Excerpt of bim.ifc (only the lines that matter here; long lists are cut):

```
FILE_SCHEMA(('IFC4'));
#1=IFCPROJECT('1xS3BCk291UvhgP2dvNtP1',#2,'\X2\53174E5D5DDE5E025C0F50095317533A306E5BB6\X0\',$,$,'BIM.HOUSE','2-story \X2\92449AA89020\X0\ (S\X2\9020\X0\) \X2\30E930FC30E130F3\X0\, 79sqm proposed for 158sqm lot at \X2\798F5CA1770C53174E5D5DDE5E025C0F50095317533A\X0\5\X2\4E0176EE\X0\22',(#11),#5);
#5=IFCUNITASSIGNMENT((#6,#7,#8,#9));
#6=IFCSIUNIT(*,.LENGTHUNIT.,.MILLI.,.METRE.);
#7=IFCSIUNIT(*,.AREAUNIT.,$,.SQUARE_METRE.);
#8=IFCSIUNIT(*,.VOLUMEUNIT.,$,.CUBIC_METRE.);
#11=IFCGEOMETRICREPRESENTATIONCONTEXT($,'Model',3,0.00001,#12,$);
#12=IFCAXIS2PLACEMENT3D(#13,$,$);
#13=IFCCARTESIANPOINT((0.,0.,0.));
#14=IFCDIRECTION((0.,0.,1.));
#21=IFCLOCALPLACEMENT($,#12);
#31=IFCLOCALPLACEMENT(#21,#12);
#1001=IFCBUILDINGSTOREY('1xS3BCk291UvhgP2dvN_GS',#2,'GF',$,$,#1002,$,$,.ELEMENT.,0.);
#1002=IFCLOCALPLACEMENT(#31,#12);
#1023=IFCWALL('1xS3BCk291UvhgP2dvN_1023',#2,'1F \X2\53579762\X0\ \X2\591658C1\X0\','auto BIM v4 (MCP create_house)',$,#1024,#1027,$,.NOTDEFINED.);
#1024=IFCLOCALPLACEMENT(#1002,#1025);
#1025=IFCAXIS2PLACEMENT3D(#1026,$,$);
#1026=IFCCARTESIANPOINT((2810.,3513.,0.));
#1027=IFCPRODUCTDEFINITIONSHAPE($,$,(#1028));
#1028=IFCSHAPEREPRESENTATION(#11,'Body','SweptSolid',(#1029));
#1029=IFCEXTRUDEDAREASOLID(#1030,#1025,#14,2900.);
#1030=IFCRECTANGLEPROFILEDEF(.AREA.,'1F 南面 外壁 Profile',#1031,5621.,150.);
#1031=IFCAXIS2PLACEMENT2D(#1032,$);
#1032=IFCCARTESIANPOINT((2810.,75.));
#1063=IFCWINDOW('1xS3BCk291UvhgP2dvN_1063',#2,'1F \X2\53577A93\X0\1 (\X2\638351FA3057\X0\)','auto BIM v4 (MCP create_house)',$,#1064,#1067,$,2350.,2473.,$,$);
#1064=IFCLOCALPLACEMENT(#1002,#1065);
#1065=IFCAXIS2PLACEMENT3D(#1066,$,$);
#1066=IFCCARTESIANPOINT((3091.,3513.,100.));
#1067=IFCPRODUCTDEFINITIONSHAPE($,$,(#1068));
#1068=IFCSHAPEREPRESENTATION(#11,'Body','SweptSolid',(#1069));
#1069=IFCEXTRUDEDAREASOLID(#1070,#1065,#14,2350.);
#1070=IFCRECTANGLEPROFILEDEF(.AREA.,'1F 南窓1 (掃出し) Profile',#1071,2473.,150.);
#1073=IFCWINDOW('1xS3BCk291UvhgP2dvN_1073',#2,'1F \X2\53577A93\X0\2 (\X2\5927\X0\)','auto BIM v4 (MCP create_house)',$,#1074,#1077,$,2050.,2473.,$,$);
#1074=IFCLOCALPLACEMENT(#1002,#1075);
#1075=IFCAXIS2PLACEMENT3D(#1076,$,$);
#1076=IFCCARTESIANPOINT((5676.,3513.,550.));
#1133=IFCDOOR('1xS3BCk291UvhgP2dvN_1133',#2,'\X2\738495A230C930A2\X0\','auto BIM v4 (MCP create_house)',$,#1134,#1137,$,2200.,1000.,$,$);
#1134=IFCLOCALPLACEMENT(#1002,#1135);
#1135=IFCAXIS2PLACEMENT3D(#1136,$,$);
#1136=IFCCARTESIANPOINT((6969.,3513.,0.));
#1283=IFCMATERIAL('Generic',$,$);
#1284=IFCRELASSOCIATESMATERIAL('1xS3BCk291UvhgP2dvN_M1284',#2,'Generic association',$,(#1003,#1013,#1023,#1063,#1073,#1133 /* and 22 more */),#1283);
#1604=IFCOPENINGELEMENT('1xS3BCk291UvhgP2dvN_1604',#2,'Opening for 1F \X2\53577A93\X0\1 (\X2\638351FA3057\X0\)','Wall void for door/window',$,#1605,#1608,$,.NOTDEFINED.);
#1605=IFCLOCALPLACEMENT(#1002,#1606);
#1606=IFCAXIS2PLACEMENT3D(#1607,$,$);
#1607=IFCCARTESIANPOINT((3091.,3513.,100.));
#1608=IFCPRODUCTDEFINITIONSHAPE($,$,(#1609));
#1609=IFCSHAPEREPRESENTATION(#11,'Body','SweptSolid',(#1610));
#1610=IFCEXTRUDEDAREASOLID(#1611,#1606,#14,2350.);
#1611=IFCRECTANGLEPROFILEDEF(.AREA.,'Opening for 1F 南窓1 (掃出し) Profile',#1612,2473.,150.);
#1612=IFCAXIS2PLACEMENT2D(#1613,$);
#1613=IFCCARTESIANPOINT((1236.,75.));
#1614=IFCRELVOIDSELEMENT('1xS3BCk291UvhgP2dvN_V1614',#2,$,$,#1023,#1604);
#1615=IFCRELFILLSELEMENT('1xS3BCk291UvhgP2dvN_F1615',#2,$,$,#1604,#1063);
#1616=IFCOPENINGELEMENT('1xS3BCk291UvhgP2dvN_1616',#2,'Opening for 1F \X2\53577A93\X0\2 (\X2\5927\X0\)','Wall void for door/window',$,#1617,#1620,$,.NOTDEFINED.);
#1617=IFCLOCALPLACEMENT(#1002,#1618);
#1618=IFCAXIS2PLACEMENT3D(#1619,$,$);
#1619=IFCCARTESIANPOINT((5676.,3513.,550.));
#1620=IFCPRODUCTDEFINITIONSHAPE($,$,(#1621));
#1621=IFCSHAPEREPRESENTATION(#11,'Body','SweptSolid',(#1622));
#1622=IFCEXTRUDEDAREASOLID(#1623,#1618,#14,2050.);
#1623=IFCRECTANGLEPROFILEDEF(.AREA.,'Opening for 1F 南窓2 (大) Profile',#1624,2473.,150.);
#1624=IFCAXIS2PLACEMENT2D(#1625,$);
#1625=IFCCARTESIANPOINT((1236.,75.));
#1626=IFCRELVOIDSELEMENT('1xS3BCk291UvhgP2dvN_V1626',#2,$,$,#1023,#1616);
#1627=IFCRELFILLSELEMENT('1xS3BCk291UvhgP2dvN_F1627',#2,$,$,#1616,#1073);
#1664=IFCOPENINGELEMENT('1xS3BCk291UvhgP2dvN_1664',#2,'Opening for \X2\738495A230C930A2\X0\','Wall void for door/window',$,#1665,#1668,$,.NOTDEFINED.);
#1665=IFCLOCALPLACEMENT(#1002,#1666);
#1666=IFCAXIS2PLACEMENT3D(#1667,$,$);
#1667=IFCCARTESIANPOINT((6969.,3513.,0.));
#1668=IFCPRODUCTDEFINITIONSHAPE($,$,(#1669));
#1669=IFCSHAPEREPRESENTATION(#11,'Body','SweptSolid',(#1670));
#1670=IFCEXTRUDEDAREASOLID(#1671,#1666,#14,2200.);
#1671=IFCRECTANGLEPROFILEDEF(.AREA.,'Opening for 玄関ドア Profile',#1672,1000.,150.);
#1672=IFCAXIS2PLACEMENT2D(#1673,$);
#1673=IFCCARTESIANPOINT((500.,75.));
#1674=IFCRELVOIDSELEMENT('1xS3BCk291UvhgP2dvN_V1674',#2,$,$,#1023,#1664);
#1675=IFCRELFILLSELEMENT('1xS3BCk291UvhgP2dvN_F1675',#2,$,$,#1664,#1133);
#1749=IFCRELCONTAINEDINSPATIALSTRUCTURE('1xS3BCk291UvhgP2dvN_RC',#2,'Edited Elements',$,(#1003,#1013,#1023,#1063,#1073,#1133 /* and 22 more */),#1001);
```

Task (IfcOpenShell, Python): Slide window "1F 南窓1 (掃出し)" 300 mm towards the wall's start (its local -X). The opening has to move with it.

```python
import ifcopenshell
import ifcopenshell.api.geometry
import ifcopenshell.util.placement

model = ifcopenshell.open("bim.ifc")

window = model.by_guid("1xS3BCk291UvhgP2dvN_1063")
opening = window.FillsVoids[0].RelatingOpeningElement
wall = opening.VoidsElements[0].RelatingBuildingElement

wall_matrix = ifcopenshell.util.placement.get_local_placement(wall.ObjectPlacement)
shift = wall_matrix[:3, 0] * -300.0
before = ifcopenshell.util.placement.get_local_placement(window.ObjectPlacement)[:3, 3].copy()

# The window is not placed relative to its opening, so move both.
for product in (opening, window):
    matrix = ifcopenshell.util.placement.get_local_placement(product.ObjectPlacement)
    matrix[:3, 3] += shift
    ifcopenshell.api.geometry.edit_object_placement(model, product=product, matrix=matrix, is_si=False)

after = ifcopenshell.util.placement.get_local_placement(window.ObjectPlacement)[:3, 3]
print("window moved by", (after - before).round(3) + 0.0)

model.write("bim-out.ifc")
```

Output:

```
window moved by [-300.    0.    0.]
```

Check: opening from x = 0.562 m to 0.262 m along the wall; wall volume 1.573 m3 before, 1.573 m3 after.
